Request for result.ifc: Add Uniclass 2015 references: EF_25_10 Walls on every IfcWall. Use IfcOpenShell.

First a look at what the model holds.

```python
import ifcopenshell

model = ifcopenshell.open("result.ifc")
print(model.schema)
print("classifications:", [c.Name for c in model.by_type("IfcClassification")])
for ifc_class in ("IfcDoor", "IfcRoof", "IfcStair", "IfcWall", "IfcWindow"):
    print(ifc_class, len(model.by_type(ifc_class)))
```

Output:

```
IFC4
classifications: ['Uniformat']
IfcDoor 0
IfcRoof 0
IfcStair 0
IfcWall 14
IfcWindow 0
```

```python
import ifcopenshell
import ifcopenshell.api.classification

model = ifcopenshell.open("result.ifc")

system = ifcopenshell.api.classification.add_classification(model, classification="Uniclass 2015")

codes = {
    "IfcWall": ("EF_25_10", "Walls"),
}
for ifc_class, (code, name) in codes.items():
    products = model.by_type(ifc_class)
    ifcopenshell.api.classification.add_reference(
        model, products=products, classification=system, identification=code, name=name
    )
    print(code, len(products))

model.write("result_rev.ifc")
```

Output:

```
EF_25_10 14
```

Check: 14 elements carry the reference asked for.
